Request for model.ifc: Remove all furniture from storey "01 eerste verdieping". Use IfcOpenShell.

First a look at what the model holds.

```python
import ifcopenshell
import ifcopenshell.util.element

model = ifcopenshell.open("model.ifc")
print(model.schema)
storey = next(s for s in model.by_type("IfcBuildingStorey") if s.Name == "01 eerste verdieping")
furniture = [e for e in ifcopenshell.util.element.get_decomposition(storey) if e.is_a("IfcFurnishingElement")]
seen = {}
for e in furniture:
    element_type = ifcopenshell.util.element.get_type(e)
    name = element_type.Name if element_type not in (None, e) else None
    seen[name] = seen.get(name, 0) + 1
for name, count in sorted(seen.items(), key=str):
    print(count, "x", name)
```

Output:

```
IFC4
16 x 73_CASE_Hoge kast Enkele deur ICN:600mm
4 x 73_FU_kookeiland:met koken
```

```python
import ifcopenshell
import ifcopenshell.api.root
import ifcopenshell.util.element

model = ifcopenshell.open("model.ifc")

storey = next(s for s in model.by_type("IfcBuildingStorey") if s.Name == "01 eerste verdieping")
furniture = [e for e in ifcopenshell.util.element.get_decomposition(storey) if e.is_a("IfcFurnishingElement")]

for e in furniture:
    ifcopenshell.api.root.remove_product(model, product=e)
print(len(furniture), "removed")

model.write("model_edited.ifc")
```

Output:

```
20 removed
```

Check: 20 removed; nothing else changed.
